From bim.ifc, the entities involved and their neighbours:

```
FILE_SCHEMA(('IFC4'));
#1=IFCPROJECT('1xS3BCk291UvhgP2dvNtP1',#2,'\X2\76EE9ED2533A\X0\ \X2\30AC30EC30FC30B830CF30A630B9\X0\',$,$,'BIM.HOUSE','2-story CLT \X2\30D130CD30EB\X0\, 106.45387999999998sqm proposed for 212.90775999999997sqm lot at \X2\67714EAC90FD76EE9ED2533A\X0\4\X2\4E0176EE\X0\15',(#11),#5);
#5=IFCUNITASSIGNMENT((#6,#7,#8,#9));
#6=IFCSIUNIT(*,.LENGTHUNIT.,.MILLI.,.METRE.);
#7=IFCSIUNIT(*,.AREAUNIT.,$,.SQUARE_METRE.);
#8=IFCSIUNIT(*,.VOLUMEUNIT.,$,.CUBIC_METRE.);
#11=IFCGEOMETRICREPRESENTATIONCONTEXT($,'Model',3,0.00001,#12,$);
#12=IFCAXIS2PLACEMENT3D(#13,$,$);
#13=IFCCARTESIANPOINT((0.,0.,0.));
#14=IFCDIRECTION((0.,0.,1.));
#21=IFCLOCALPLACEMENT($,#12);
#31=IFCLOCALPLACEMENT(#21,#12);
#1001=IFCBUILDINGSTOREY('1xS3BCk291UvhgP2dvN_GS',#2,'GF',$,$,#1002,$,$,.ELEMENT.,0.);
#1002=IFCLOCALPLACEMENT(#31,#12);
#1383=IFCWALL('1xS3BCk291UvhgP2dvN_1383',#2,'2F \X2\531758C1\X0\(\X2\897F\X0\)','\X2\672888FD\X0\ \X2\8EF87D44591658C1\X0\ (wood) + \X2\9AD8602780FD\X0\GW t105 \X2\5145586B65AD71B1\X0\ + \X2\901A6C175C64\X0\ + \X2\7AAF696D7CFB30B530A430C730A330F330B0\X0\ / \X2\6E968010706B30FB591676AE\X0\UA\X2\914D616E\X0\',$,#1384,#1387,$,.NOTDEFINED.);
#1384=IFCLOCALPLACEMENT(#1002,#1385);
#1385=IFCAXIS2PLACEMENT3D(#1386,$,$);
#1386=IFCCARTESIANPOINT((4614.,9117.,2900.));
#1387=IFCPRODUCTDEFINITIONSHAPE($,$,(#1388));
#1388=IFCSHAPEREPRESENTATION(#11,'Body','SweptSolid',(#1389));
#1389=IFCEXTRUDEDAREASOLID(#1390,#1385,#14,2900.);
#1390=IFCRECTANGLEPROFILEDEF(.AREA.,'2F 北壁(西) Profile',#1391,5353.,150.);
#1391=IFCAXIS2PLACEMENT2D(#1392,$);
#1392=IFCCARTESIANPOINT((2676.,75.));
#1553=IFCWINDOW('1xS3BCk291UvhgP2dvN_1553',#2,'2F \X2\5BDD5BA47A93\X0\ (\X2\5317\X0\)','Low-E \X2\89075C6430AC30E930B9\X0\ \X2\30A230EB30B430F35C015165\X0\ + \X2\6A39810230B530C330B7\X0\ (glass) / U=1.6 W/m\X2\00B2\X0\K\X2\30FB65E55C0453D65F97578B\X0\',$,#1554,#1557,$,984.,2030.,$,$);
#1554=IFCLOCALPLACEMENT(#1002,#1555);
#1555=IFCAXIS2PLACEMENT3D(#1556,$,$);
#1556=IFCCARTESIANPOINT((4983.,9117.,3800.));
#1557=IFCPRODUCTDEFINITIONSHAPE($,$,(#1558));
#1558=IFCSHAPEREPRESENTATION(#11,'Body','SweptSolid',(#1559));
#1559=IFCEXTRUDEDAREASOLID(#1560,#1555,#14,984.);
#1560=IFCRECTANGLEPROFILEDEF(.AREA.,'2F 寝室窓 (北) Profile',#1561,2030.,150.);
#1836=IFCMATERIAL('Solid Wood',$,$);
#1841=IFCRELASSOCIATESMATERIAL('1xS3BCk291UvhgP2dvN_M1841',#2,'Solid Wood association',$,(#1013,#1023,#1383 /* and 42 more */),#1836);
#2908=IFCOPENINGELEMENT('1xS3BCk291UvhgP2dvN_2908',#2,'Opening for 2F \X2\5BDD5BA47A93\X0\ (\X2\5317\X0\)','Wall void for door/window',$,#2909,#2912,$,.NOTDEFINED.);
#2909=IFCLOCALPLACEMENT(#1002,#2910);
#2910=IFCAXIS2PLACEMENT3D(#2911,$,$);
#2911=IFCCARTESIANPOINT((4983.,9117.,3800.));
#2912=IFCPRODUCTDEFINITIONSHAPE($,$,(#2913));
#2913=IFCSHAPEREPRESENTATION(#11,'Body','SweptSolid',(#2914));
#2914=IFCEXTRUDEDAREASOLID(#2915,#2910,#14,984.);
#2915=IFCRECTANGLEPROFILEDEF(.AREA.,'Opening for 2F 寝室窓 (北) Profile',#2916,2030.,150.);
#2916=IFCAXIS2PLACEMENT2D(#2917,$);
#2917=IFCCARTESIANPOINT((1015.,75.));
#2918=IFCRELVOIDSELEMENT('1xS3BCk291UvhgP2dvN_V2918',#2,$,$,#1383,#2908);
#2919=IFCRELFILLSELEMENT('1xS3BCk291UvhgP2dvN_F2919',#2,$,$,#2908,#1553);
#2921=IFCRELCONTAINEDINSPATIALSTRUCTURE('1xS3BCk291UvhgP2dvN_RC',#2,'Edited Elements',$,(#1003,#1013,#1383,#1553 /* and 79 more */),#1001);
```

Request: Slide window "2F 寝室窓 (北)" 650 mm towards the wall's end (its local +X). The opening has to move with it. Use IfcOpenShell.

```python
import ifcopenshell
import ifcopenshell.api.geometry
import ifcopenshell.util.placement
import ifcopenshell.util.unit

model = ifcopenshell.open("bim.ifc")
unit_scale = ifcopenshell.util.unit.calculate_unit_scale(model)

window = model.by_id(1553)
opening = window.FillsVoids[0].RelatingOpeningElement
wall = opening.VoidsElements[0].RelatingBuildingElement

wall_matrix = ifcopenshell.util.placement.get_local_placement(wall.ObjectPlacement)
shift = wall_matrix[:3, 0] * 0.65 / unit_scale
before = ifcopenshell.util.placement.get_local_placement(window.ObjectPlacement)[:3, 3].copy()

# The window is not placed relative to its opening, so move both.
for product in (opening, window):
    matrix = ifcopenshell.util.placement.get_local_placement(product.ObjectPlacement)
    matrix[:3, 3] += shift
    ifcopenshell.api.geometry.edit_object_placement(model, product=product, matrix=matrix, is_si=False)

after = ifcopenshell.util.placement.get_local_placement(window.ObjectPlacement)[:3, 3]
print("window moved by", (after - before).round(3) + 0.0)

model.write("bim_rev.ifc")
```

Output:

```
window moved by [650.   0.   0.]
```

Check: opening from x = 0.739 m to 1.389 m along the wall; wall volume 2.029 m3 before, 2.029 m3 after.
